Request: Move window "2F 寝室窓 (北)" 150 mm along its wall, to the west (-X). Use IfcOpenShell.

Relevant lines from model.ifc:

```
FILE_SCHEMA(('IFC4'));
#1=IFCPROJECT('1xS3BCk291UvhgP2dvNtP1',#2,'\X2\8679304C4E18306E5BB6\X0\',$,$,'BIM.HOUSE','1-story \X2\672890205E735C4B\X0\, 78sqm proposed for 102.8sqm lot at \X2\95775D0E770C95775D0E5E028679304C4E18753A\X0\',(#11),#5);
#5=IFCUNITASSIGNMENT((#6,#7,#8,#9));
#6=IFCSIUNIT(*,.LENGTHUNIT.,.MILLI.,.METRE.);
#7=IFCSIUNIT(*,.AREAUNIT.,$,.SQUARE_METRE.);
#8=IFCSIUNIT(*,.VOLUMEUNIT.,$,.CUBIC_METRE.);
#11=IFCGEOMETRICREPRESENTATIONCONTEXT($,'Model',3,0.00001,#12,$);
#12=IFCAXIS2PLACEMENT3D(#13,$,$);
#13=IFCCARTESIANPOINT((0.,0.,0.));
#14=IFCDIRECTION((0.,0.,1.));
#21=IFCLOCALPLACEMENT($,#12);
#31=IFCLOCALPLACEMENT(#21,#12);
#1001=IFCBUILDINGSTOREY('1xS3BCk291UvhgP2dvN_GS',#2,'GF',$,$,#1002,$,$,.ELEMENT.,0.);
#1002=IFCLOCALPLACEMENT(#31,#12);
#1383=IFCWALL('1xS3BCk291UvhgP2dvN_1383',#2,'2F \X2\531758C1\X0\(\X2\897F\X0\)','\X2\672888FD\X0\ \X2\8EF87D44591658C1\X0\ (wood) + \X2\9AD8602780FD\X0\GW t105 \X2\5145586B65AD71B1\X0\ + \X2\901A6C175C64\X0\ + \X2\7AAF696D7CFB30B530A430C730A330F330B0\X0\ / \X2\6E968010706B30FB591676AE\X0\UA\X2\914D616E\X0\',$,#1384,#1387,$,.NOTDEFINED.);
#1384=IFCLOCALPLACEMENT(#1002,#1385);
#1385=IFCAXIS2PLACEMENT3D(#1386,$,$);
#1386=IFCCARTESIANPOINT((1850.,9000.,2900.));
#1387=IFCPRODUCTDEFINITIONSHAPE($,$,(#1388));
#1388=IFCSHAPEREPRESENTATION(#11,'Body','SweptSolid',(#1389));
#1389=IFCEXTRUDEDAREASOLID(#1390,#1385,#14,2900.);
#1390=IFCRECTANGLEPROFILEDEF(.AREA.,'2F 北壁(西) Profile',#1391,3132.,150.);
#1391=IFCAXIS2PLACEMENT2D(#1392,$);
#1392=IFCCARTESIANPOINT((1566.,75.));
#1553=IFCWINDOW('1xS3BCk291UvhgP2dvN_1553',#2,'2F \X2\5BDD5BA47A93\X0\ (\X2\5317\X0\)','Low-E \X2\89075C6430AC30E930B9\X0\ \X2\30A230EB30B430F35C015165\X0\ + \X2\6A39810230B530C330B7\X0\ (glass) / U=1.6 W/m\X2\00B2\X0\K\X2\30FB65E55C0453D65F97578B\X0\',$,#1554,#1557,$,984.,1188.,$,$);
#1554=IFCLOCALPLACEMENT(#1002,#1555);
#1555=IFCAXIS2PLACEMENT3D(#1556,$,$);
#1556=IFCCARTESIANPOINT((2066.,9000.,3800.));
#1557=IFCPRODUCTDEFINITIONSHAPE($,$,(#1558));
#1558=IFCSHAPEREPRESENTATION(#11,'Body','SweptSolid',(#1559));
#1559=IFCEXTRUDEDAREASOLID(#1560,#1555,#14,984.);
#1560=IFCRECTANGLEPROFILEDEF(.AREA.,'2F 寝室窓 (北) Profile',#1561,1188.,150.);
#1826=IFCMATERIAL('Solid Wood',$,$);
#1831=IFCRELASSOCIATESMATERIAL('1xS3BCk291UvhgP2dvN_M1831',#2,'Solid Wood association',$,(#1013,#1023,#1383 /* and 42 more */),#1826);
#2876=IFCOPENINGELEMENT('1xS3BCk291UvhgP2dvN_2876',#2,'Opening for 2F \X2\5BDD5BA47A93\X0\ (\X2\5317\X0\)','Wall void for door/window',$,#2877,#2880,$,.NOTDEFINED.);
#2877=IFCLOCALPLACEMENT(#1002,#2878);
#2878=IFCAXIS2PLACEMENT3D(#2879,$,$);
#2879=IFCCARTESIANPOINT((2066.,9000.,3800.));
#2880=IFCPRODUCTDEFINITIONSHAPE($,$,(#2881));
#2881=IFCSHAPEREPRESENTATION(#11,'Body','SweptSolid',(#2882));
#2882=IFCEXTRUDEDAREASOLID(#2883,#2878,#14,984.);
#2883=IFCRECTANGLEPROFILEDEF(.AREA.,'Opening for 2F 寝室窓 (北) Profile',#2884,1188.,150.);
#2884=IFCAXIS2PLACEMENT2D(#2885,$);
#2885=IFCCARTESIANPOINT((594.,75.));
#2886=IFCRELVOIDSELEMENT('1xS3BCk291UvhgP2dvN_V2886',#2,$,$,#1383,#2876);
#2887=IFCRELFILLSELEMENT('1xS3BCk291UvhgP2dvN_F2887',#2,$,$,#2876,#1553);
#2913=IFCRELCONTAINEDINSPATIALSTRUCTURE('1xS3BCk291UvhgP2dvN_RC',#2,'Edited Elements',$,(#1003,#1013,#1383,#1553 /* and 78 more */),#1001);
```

```python
import ifcopenshell
import ifcopenshell.api.geometry
import ifcopenshell.util.placement
import ifcopenshell.util.unit

model = ifcopenshell.open("model.ifc")
unit_scale = ifcopenshell.util.unit.calculate_unit_scale(model)

window = model.by_guid("1xS3BCk291UvhgP2dvN_1553")
opening = window.FillsVoids[0].RelatingOpeningElement
wall = opening.VoidsElements[0].RelatingBuildingElement

wall_matrix = ifcopenshell.util.placement.get_local_placement(wall.ObjectPlacement)
shift = wall_matrix[:3, 0] * -0.15 / unit_scale
before = ifcopenshell.util.placement.get_local_placement(window.ObjectPlacement)[:3, 3].copy()

# The window is not placed relative to its opening, so move both.
for product in (opening, window):
    matrix = ifcopenshell.util.placement.get_local_placement(product.ObjectPlacement)
    matrix[:3, 3] += shift
    ifcopenshell.api.geometry.edit_object_placement(model, product=product, matrix=matrix, is_si=False)

after = ifcopenshell.util.placement.get_local_placement(window.ObjectPlacement)[:3, 3]
print("window moved by", (after - before).round(3) + 0.0)

model.write("model_edited.ifc")
```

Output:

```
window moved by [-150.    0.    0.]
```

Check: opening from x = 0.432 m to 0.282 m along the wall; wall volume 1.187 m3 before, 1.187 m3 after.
